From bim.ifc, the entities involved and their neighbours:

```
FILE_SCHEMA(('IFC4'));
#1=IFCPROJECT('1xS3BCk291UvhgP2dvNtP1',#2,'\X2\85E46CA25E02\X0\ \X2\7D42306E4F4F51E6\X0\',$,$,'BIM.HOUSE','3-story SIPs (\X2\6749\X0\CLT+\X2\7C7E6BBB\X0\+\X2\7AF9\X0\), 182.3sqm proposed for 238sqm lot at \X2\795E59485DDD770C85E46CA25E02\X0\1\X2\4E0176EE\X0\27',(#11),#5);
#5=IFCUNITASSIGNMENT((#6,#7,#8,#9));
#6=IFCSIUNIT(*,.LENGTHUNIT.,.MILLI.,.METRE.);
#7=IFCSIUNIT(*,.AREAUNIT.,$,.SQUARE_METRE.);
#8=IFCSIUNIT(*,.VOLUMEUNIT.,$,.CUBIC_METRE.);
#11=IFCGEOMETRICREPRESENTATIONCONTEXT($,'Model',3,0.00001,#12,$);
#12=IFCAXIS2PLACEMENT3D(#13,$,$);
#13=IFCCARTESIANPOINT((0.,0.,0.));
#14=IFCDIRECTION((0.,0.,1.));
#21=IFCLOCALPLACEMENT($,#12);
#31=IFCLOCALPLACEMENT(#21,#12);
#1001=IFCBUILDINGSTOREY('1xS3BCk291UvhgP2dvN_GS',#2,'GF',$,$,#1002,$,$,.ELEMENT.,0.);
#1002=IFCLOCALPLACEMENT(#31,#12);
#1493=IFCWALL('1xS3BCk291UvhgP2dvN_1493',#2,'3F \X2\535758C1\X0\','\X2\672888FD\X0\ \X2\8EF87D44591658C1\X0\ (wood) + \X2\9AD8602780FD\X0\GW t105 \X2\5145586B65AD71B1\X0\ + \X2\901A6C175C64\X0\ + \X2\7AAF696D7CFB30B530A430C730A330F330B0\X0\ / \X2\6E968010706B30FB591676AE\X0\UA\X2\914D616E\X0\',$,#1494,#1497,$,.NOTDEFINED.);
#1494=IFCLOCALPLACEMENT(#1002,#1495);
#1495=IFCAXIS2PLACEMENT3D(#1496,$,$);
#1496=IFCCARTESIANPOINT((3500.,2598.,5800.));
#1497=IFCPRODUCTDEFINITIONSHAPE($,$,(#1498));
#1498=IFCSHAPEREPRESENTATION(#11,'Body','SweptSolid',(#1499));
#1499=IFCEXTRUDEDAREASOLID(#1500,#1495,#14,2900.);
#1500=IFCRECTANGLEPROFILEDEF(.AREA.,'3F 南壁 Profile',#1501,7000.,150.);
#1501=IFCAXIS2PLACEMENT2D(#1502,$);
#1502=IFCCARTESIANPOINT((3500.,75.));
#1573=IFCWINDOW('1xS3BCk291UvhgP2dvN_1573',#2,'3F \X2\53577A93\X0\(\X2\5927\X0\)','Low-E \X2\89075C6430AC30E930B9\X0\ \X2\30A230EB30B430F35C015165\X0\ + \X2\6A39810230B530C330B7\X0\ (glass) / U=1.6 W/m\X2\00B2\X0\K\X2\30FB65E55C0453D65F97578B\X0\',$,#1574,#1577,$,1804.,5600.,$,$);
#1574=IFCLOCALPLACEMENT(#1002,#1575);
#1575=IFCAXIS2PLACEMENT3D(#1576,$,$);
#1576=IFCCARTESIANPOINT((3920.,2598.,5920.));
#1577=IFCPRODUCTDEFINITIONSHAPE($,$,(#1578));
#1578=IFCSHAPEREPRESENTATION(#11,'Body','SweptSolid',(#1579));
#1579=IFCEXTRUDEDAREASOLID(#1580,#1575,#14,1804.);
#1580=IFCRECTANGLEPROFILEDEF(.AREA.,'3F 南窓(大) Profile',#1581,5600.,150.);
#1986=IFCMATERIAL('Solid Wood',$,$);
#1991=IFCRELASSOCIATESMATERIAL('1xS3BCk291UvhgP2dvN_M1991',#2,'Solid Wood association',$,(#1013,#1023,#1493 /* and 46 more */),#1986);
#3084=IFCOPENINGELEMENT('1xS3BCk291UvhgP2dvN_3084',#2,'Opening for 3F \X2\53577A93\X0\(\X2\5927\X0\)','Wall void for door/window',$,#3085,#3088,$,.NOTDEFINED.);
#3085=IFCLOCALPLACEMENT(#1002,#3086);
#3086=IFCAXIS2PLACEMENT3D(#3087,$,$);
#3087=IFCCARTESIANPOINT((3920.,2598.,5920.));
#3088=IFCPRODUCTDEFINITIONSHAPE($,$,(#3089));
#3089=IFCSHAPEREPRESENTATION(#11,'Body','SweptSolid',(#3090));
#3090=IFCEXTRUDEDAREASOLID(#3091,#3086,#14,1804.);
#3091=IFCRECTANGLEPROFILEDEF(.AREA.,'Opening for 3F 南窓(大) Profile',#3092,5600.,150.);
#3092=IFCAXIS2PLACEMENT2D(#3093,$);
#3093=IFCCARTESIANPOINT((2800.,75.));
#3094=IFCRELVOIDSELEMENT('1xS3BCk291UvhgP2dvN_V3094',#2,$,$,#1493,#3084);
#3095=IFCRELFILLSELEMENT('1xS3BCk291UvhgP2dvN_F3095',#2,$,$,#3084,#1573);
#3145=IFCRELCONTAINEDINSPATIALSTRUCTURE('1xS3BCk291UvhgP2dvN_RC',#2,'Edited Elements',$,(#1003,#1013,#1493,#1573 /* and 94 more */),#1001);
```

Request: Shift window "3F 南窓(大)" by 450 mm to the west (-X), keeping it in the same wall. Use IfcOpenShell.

```python
import ifcopenshell
import ifcopenshell.api.geometry
import ifcopenshell.util.placement
import ifcopenshell.util.unit

model = ifcopenshell.open("bim.ifc")
unit_scale = ifcopenshell.util.unit.calculate_unit_scale(model)

window = model.by_id(1573)
opening = window.FillsVoids[0].RelatingOpeningElement
wall = opening.VoidsElements[0].RelatingBuildingElement

wall_matrix = ifcopenshell.util.placement.get_local_placement(wall.ObjectPlacement)
shift = wall_matrix[:3, 0] * -0.45 / unit_scale
before = ifcopenshell.util.placement.get_local_placement(window.ObjectPlacement)[:3, 3].copy()

# The window is not placed relative to its opening, so move both.
for product in (opening, window):
    matrix = ifcopenshell.util.placement.get_local_placement(product.ObjectPlacement)
    matrix[:3, 3] += shift
    ifcopenshell.api.geometry.edit_object_placement(model, product=product, matrix=matrix, is_si=False)

after = ifcopenshell.util.placement.get_local_placement(window.ObjectPlacement)[:3, 3]
print("window moved by", (after - before).round(3) + 0.0)

model.write("bim_rev.ifc")
```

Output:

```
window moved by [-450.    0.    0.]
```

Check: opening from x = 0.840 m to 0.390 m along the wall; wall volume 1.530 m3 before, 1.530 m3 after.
